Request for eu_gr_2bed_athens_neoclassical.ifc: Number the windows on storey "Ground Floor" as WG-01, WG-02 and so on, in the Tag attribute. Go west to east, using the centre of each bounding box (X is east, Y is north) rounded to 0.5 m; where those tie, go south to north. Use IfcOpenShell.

First a look at what the model holds.

```python
import ifcopenshell
import ifcopenshell.util.element
import ifcopenshell.util.placement

model = ifcopenshell.open("eu_gr_2bed_athens_neoclassical.ifc")
print(model.schema)
storey = next(s for s in model.by_type("IfcBuildingStorey") if s.Name == "Ground Floor")
windows = [e for e in ifcopenshell.util.element.get_decomposition(storey) if e.is_a("IfcWindow")]
for e in sorted(windows, key=lambda e: e.id()):
    origin = ifcopenshell.util.placement.get_local_placement(e.ObjectPlacement)[:3, 3]
    print(e.id(), e.Tag, e.Name, origin.round(2) + 0.0, sep=" | ")
```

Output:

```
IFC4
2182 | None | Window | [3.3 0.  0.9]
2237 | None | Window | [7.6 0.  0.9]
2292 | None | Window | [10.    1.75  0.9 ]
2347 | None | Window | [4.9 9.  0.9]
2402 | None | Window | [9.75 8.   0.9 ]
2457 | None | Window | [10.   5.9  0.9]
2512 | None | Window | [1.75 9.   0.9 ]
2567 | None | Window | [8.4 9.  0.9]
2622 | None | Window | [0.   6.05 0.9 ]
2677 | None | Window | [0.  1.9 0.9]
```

```python
import ifcopenshell
import ifcopenshell.geom
import ifcopenshell.util.element
import ifcopenshell.util.shape

model = ifcopenshell.open("eu_gr_2bed_athens_neoclassical.ifc")
settings = ifcopenshell.geom.settings()
settings.set("use-world-coords", True)


def centre(element):
    shape = ifcopenshell.geom.create_shape(settings, element)
    return ifcopenshell.util.shape.get_bbox_centroid(shape.geometry)


storey = next(s for s in model.by_type("IfcBuildingStorey") if s.Name == "Ground Floor")
windows = [e for e in ifcopenshell.util.element.get_decomposition(storey) if e.is_a("IfcWindow")]

# Insertion points can sit at a corner or the storey origin, so sort by the geometry (in metres).
centres = {e: centre(e) for e in windows}
windows.sort(key=lambda e: (round(centres[e][0] / 0.5), centres[e][1]))

for i, e in enumerate(windows, start=1):
    number = f"WG-{i:02d}"
    e.Tag = number
    print(e.id(), number)

model.write("eu_gr_2bed_athens_neoclassical_updated.ifc")
```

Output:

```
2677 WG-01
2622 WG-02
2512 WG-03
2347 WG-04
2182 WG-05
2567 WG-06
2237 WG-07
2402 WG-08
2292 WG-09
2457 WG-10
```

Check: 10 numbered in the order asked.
